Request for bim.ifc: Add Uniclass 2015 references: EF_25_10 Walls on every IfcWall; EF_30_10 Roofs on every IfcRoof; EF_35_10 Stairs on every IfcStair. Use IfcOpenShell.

First a look at what the model holds.

```python
import ifcopenshell

model = ifcopenshell.open("bim.ifc")
print(model.schema)
print("classifications:", [c.Name for c in model.by_type("IfcClassification")])
for ifc_class in ("IfcDoor", "IfcRoof", "IfcStair", "IfcWall", "IfcWindow"):
    print(ifc_class, len(model.by_type(ifc_class)))
```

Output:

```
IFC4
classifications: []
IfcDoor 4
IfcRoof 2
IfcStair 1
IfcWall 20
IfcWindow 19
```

```python
import ifcopenshell
import ifcopenshell.api.classification

model = ifcopenshell.open("bim.ifc")

system = ifcopenshell.api.classification.add_classification(model, classification="Uniclass 2015")

codes = {
    "IfcWall": ("EF_25_10", "Walls"),
    "IfcRoof": ("EF_30_10", "Roofs"),
    "IfcStair": ("EF_35_10", "Stairs"),
}
for ifc_class, (code, name) in codes.items():
    products = model.by_type(ifc_class)
    ifcopenshell.api.classification.add_reference(
        model, products=products, classification=system, identification=code, name=name
    )
    print(code, len(products))

model.write("bim_v2.ifc")
```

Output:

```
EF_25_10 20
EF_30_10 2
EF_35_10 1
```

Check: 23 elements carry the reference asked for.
